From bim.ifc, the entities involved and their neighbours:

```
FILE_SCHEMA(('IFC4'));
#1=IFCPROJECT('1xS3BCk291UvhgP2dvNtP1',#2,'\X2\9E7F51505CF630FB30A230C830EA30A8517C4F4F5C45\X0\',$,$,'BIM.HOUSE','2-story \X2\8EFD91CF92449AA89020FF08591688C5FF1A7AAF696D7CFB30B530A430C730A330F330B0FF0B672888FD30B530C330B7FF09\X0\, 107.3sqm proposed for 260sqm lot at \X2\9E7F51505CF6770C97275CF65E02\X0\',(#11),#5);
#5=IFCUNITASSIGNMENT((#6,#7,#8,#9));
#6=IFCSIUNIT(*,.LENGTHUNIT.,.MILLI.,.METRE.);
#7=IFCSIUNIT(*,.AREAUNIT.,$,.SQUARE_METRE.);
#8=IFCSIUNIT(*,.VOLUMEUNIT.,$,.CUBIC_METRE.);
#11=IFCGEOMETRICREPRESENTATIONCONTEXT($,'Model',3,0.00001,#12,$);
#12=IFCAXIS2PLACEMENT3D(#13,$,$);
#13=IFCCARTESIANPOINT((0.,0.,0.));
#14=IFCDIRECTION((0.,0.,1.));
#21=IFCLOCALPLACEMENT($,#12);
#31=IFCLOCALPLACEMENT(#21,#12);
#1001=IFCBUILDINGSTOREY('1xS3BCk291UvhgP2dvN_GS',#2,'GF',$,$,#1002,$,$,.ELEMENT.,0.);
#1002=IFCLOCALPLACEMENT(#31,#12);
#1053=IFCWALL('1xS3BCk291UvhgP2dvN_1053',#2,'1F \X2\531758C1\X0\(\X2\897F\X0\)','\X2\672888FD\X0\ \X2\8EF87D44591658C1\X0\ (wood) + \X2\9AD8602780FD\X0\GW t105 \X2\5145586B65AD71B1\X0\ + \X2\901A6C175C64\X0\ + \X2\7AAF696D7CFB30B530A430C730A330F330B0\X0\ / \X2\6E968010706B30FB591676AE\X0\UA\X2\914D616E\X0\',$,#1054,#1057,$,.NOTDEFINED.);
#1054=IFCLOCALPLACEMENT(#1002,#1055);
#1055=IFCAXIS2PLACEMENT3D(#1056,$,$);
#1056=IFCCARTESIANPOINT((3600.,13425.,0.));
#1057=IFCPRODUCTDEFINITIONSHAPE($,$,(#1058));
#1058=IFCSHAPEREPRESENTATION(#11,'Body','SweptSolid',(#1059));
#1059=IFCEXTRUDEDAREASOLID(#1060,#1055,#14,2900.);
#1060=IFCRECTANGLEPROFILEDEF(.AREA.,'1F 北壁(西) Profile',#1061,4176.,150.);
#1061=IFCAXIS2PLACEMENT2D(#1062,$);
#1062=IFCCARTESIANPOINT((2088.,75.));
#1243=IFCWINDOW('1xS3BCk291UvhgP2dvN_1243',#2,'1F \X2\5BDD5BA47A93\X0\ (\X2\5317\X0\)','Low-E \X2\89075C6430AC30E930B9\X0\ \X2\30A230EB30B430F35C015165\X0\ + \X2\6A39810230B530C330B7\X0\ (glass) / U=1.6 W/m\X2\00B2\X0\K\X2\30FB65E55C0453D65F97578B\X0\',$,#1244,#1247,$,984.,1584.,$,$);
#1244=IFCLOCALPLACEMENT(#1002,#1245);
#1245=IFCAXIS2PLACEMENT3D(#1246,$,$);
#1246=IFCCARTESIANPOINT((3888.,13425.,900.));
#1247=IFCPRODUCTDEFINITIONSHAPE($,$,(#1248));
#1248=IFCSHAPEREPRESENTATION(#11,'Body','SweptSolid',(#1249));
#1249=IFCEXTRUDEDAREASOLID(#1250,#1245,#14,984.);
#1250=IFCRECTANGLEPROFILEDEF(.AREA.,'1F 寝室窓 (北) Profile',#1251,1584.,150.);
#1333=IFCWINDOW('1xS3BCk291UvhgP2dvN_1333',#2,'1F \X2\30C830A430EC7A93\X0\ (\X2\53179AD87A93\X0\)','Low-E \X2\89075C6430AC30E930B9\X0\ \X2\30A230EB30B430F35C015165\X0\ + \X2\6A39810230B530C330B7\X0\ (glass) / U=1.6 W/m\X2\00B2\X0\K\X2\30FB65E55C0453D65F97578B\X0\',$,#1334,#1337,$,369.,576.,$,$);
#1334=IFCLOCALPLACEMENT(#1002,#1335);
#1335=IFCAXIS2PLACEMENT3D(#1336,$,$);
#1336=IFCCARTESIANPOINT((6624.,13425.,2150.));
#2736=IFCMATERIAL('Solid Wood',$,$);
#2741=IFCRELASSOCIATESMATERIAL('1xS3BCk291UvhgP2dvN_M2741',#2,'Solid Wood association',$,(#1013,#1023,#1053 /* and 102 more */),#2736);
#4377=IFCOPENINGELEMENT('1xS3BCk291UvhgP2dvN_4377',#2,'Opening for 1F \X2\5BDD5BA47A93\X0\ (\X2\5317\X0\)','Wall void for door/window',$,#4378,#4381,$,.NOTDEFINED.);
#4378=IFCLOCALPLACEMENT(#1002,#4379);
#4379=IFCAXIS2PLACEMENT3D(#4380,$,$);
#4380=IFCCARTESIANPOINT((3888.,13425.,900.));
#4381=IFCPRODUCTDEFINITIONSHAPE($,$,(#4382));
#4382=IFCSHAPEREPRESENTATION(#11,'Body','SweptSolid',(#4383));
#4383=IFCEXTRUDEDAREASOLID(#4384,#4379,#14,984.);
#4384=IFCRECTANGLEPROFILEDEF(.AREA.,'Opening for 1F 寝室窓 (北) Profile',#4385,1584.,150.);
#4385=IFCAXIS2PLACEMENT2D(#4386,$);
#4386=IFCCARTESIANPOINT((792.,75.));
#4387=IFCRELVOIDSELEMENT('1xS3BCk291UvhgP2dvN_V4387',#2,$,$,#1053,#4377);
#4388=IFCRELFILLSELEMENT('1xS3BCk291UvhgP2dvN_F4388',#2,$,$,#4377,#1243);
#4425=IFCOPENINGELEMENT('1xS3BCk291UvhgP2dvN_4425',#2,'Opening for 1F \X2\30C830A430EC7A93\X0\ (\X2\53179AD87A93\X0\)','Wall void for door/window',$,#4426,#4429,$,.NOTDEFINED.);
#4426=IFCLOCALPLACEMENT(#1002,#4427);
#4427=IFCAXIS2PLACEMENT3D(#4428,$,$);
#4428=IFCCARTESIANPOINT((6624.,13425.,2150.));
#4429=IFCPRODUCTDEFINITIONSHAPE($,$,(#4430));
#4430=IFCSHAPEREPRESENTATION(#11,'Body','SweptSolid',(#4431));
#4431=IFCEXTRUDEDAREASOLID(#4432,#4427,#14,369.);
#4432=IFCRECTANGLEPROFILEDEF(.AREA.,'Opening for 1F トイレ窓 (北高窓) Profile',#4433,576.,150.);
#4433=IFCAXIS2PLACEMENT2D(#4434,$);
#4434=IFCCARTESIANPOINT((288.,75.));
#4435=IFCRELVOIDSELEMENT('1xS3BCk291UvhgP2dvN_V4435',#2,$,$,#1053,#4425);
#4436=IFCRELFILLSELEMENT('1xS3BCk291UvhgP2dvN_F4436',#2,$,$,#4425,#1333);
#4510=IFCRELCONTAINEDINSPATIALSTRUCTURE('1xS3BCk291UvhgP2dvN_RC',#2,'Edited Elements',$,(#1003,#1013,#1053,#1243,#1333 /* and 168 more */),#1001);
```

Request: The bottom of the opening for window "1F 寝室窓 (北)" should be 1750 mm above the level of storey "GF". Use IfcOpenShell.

```python
import numpy as np
import ifcopenshell
import ifcopenshell.api.geometry
import ifcopenshell.geom
import ifcopenshell.util.element
import ifcopenshell.util.placement
import ifcopenshell.util.shape
import ifcopenshell.util.unit

model = ifcopenshell.open("bim.ifc")
unit_scale = ifcopenshell.util.unit.calculate_unit_scale(model)

window = model.by_id(1243)
opening = window.FillsVoids[0].RelatingOpeningElement
storey = ifcopenshell.util.element.get_container(window, ifc_class="IfcBuildingStorey")
level = ifcopenshell.util.placement.get_local_placement(storey.ObjectPlacement)[2, 3]

# The opening's origin need not be at the sill, so measure its lowest point.
shape = ifcopenshell.geom.create_shape(ifcopenshell.geom.settings(), opening)
bottom = ifcopenshell.util.shape.get_shape_bottom_elevation(shape, shape.geometry) / unit_scale
dz = level + 1750.0 - bottom

shift = np.array([0.0, 0.0, dz])
# The window is not placed relative to its opening, so move both.
for product in (opening, window):
    matrix = ifcopenshell.util.placement.get_local_placement(product.ObjectPlacement)
    matrix[:3, 3] += shift
    ifcopenshell.api.geometry.edit_object_placement(model, product=product, matrix=matrix, is_si=False)

print(f"moved by {dz * unit_scale:+.3f} m")

model.write("bim_v2.ifc")
```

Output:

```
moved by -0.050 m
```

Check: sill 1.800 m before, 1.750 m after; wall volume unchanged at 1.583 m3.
